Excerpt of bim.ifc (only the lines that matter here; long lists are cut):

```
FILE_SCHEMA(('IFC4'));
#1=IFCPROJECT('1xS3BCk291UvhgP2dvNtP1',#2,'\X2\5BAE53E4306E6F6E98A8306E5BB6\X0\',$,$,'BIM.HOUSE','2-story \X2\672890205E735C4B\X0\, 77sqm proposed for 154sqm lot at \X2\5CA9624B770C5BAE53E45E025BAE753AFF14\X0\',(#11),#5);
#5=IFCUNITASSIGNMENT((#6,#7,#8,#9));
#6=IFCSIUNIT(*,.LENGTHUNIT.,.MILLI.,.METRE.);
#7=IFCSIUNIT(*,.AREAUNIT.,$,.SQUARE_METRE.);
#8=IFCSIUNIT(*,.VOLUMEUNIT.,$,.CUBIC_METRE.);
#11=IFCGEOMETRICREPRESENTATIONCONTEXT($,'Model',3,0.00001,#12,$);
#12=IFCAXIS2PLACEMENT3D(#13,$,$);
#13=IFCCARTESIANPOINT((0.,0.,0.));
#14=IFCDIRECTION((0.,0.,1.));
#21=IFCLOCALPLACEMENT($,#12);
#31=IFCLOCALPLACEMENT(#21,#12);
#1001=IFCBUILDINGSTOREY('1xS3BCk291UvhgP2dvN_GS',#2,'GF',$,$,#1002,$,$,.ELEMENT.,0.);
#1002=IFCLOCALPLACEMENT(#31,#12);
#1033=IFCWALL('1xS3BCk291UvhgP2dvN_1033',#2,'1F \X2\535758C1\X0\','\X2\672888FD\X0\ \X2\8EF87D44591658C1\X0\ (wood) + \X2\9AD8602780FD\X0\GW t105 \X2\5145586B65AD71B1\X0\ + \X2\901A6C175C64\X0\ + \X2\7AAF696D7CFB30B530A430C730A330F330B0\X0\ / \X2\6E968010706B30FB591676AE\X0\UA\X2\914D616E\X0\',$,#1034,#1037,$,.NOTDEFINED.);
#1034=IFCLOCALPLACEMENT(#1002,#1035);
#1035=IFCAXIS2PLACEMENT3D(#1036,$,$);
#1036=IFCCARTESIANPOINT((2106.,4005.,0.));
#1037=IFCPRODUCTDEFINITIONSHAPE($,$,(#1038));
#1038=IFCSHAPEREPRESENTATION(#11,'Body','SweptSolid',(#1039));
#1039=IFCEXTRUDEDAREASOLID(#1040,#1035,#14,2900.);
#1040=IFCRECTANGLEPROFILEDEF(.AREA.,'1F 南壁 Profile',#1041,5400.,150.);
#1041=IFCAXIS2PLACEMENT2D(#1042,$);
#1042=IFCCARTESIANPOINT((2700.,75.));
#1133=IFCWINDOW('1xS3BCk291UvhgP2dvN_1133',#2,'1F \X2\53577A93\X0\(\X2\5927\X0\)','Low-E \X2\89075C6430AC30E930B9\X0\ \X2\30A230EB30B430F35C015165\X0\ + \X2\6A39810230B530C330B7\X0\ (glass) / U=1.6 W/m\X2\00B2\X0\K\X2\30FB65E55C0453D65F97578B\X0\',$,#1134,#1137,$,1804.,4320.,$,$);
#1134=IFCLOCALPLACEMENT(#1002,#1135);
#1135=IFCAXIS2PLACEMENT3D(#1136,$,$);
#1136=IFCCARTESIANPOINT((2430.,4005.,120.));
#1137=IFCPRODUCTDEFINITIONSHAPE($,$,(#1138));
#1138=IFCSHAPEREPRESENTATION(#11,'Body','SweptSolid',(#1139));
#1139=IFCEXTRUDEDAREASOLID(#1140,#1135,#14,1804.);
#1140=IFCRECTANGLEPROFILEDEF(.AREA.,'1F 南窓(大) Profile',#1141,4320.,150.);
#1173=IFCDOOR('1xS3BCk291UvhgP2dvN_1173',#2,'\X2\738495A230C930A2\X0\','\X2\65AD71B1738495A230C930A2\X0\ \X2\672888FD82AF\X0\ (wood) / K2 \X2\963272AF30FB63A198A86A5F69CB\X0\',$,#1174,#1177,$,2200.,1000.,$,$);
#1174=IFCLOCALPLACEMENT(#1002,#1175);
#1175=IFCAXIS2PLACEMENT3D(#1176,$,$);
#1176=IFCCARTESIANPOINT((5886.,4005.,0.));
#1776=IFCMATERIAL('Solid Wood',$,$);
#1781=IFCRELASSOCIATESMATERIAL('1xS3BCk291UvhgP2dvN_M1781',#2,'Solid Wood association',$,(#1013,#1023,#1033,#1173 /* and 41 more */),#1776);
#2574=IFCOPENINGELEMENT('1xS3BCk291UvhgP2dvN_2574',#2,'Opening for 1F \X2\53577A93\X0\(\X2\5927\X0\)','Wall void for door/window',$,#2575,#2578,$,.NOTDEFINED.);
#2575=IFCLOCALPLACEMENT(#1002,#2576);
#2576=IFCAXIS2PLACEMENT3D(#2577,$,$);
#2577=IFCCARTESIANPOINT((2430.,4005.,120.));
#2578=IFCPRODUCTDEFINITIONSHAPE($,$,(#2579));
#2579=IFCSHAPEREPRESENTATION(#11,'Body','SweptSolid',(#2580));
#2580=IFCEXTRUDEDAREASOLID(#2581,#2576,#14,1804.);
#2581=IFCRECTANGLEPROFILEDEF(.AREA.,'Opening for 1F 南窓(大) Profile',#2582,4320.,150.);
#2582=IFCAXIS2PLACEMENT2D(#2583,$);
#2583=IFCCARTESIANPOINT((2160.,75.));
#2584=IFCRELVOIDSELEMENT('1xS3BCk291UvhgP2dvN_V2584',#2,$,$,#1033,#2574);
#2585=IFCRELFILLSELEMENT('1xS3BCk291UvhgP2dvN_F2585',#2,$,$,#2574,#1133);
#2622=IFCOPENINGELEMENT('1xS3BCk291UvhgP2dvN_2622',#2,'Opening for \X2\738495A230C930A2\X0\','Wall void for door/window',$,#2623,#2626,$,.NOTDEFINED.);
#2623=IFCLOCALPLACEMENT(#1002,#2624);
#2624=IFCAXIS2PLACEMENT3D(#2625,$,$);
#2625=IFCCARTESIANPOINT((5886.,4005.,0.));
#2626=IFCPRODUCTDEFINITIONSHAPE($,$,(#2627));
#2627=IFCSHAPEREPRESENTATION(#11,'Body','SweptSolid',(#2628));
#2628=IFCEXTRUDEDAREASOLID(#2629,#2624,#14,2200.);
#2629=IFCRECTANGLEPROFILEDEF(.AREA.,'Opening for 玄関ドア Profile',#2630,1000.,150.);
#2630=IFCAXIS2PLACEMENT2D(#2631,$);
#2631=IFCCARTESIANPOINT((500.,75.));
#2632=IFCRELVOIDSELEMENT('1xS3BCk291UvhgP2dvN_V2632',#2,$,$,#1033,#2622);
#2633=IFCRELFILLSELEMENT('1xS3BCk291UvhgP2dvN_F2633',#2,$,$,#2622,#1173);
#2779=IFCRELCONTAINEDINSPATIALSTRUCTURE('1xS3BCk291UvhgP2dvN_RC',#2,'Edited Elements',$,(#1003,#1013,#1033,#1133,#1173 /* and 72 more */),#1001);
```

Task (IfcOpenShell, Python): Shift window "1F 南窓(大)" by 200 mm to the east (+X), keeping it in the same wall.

```python
import ifcopenshell
import ifcopenshell.api.geometry
import ifcopenshell.util.placement
import ifcopenshell.util.unit

model = ifcopenshell.open("bim.ifc")
unit_scale = ifcopenshell.util.unit.calculate_unit_scale(model)

window = model.by_guid("1xS3BCk291UvhgP2dvN_1133")
opening = window.FillsVoids[0].RelatingOpeningElement
wall = opening.VoidsElements[0].RelatingBuildingElement

wall_matrix = ifcopenshell.util.placement.get_local_placement(wall.ObjectPlacement)
shift = wall_matrix[:3, 0] * 0.2 / unit_scale
before = ifcopenshell.util.placement.get_local_placement(window.ObjectPlacement)[:3, 3].copy()

# The window is not placed relative to its opening, so move both.
for product in (opening, window):
    matrix = ifcopenshell.util.placement.get_local_placement(product.ObjectPlacement)
    matrix[:3, 3] += shift
    ifcopenshell.api.geometry.edit_object_placement(model, product=product, matrix=matrix, is_si=False)

after = ifcopenshell.util.placement.get_local_placement(window.ObjectPlacement)[:3, 3]
print("window moved by", (after - before).round(3) + 0.0)

model.write("bim_v2.ifc")
```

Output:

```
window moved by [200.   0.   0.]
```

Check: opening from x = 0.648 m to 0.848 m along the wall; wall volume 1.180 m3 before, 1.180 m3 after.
